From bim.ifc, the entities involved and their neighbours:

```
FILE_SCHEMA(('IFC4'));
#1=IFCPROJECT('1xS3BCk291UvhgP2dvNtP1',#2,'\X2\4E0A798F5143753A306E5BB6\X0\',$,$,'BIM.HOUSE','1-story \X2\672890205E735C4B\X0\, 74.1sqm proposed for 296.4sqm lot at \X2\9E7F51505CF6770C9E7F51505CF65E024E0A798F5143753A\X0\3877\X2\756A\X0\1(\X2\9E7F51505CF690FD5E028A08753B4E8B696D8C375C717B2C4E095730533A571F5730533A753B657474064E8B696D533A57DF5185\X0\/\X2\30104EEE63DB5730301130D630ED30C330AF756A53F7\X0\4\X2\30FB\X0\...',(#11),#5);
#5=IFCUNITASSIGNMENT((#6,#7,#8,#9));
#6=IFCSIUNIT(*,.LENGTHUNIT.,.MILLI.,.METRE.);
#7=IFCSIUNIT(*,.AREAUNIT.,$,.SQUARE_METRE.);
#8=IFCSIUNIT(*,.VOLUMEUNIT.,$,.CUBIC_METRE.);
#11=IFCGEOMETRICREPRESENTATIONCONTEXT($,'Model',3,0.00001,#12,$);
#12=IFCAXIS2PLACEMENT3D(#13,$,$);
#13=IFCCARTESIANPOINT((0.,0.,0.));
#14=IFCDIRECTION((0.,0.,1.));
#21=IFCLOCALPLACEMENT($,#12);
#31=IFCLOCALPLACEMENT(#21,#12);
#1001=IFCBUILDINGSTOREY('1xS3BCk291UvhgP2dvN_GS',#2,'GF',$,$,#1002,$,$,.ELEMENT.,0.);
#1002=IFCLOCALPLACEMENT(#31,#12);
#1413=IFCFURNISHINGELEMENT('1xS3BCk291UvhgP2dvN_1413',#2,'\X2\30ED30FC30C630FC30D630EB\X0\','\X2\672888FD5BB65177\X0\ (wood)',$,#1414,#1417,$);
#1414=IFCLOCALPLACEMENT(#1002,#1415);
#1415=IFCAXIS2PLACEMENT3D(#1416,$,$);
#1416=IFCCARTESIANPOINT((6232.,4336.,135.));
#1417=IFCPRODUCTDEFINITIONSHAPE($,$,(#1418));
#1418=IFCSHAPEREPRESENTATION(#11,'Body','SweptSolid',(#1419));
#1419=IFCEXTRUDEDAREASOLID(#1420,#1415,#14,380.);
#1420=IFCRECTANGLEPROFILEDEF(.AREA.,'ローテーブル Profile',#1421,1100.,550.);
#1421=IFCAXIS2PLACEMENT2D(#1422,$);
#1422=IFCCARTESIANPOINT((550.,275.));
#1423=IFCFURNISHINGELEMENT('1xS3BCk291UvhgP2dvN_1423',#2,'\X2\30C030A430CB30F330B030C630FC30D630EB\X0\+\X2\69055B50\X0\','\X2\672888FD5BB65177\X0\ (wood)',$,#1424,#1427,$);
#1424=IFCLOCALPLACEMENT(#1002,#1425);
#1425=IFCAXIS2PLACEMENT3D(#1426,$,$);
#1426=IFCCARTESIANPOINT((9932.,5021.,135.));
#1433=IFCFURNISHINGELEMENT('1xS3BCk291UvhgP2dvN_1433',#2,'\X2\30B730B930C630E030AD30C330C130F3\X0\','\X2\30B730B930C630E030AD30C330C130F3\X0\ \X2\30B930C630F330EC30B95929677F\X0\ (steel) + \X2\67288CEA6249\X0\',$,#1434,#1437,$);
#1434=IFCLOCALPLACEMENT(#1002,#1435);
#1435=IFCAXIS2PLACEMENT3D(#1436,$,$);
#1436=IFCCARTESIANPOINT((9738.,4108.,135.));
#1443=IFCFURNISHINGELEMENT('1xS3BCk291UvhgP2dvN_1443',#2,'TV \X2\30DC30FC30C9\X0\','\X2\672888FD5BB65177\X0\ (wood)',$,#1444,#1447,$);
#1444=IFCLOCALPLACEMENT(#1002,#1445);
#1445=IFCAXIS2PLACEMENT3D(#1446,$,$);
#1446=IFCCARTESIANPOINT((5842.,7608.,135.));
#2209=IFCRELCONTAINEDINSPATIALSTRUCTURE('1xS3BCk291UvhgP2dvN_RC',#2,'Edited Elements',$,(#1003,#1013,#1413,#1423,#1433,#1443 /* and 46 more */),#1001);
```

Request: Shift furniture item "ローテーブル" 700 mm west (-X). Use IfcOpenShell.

```python
import ifcopenshell
import ifcopenshell.api.geometry
import ifcopenshell.util.placement
import ifcopenshell.util.unit

model = ifcopenshell.open("bim.ifc")
unit_scale = ifcopenshell.util.unit.calculate_unit_scale(model)

item = model.by_guid("1xS3BCk291UvhgP2dvN_1413")
matrix = ifcopenshell.util.placement.get_local_placement(item.ObjectPlacement)
matrix[0, 3] -= 0.7 / unit_scale
ifcopenshell.api.geometry.edit_object_placement(model, product=item, matrix=matrix, is_si=False)

print(ifcopenshell.util.placement.get_local_placement(item.ObjectPlacement).round(3) + 0.0)

model.write("bim_updated.ifc")
```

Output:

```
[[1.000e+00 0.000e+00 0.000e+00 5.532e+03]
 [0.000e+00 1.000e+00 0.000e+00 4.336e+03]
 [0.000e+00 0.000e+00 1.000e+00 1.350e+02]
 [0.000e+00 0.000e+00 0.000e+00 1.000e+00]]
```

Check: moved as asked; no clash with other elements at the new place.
